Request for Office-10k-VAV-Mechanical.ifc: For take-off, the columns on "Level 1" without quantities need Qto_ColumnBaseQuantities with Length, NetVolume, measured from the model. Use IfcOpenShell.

First a look at what the model holds.

```python
import ifcopenshell
import ifcopenshell.util.element
import ifcopenshell.util.unit

model = ifcopenshell.open("Office-10k-VAV-Mechanical.ifc")
print(model.schema)
for unit_type in ("LENGTHUNIT", "AREAUNIT", "VOLUMEUNIT"):
    print(unit_type, ifcopenshell.util.unit.calculate_unit_scale(model, unit_type))
storey = next(s for s in model.by_type("IfcBuildingStorey") if s.Name == "Level 1")
columns = [e for e in ifcopenshell.util.element.get_decomposition(storey) if e.is_a("IfcColumn")]
for e in sorted(columns, key=lambda e: e.id()):
    print(e.id(), e.is_a(), e.Name, list(ifcopenshell.util.element.get_psets(e, qtos_only=True)), sep=" | ")
```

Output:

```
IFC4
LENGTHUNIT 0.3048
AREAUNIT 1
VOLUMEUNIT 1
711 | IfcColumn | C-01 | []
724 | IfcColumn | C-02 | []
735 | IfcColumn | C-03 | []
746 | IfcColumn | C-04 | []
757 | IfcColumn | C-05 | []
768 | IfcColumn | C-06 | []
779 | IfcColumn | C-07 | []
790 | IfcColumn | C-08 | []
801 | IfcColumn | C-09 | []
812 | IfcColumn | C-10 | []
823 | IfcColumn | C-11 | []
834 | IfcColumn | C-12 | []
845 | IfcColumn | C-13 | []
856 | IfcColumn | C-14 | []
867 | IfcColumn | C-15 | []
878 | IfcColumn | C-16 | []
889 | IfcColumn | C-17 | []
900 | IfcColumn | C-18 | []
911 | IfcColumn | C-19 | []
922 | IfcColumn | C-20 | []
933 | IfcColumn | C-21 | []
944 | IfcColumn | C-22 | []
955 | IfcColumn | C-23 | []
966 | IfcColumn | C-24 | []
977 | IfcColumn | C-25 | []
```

```python
import ifcopenshell
import ifcopenshell.api.pset
import ifcopenshell.geom
import ifcopenshell.util.element
import ifcopenshell.util.shape
import ifcopenshell.util.unit

model = ifcopenshell.open("Office-10k-VAV-Mechanical.ifc")
unit_scale = ifcopenshell.util.unit.calculate_unit_scale(model)
volume_scale = ifcopenshell.util.unit.calculate_unit_scale(model, "VOLUMEUNIT")
settings = ifcopenshell.geom.settings()

storey = next(s for s in model.by_type("IfcBuildingStorey") if s.Name == "Level 1")
columns = [e for e in ifcopenshell.util.element.get_decomposition(storey) if e.is_a("IfcColumn")]

for e in sorted(columns, key=lambda e: e.id()):
    if ifcopenshell.util.element.get_psets(e, qtos_only=True, should_inherit=False):
        continue
    # Geometry comes back in metres, in the element's own axes.
    shape = ifcopenshell.geom.create_shape(settings, e)
    values = {
        "Length": ifcopenshell.util.shape.get_z(shape.geometry) / unit_scale,
        "NetVolume": ifcopenshell.util.shape.get_volume(shape.geometry) / volume_scale,
    }
    qto = ifcopenshell.api.pset.add_qto(model, product=e, name="Qto_ColumnBaseQuantities")
    ifcopenshell.api.pset.edit_qto(model, qto=qto, properties=values)
    print(e.id(), {k: round(v, 3) for k, v in values.items()})

model.write("Office-10k-VAV-Mechanical_updated.ifc")
```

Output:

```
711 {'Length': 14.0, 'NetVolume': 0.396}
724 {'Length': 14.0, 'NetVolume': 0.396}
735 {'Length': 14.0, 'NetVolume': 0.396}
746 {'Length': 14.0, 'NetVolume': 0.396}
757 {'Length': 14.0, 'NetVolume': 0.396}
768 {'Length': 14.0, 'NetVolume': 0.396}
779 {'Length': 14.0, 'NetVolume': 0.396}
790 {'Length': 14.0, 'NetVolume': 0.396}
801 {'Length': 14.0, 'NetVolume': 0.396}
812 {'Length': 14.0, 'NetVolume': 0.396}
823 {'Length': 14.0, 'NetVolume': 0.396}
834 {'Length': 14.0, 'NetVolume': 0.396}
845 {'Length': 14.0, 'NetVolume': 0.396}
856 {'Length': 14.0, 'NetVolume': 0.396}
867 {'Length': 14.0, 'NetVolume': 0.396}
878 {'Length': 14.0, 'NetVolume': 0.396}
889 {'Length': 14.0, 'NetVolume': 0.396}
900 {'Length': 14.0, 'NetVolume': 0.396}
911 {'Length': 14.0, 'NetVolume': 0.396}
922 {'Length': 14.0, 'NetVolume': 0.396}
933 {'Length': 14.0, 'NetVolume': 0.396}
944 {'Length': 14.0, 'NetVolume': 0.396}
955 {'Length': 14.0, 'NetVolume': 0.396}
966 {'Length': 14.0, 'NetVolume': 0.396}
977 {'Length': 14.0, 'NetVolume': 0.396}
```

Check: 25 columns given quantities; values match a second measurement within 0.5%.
